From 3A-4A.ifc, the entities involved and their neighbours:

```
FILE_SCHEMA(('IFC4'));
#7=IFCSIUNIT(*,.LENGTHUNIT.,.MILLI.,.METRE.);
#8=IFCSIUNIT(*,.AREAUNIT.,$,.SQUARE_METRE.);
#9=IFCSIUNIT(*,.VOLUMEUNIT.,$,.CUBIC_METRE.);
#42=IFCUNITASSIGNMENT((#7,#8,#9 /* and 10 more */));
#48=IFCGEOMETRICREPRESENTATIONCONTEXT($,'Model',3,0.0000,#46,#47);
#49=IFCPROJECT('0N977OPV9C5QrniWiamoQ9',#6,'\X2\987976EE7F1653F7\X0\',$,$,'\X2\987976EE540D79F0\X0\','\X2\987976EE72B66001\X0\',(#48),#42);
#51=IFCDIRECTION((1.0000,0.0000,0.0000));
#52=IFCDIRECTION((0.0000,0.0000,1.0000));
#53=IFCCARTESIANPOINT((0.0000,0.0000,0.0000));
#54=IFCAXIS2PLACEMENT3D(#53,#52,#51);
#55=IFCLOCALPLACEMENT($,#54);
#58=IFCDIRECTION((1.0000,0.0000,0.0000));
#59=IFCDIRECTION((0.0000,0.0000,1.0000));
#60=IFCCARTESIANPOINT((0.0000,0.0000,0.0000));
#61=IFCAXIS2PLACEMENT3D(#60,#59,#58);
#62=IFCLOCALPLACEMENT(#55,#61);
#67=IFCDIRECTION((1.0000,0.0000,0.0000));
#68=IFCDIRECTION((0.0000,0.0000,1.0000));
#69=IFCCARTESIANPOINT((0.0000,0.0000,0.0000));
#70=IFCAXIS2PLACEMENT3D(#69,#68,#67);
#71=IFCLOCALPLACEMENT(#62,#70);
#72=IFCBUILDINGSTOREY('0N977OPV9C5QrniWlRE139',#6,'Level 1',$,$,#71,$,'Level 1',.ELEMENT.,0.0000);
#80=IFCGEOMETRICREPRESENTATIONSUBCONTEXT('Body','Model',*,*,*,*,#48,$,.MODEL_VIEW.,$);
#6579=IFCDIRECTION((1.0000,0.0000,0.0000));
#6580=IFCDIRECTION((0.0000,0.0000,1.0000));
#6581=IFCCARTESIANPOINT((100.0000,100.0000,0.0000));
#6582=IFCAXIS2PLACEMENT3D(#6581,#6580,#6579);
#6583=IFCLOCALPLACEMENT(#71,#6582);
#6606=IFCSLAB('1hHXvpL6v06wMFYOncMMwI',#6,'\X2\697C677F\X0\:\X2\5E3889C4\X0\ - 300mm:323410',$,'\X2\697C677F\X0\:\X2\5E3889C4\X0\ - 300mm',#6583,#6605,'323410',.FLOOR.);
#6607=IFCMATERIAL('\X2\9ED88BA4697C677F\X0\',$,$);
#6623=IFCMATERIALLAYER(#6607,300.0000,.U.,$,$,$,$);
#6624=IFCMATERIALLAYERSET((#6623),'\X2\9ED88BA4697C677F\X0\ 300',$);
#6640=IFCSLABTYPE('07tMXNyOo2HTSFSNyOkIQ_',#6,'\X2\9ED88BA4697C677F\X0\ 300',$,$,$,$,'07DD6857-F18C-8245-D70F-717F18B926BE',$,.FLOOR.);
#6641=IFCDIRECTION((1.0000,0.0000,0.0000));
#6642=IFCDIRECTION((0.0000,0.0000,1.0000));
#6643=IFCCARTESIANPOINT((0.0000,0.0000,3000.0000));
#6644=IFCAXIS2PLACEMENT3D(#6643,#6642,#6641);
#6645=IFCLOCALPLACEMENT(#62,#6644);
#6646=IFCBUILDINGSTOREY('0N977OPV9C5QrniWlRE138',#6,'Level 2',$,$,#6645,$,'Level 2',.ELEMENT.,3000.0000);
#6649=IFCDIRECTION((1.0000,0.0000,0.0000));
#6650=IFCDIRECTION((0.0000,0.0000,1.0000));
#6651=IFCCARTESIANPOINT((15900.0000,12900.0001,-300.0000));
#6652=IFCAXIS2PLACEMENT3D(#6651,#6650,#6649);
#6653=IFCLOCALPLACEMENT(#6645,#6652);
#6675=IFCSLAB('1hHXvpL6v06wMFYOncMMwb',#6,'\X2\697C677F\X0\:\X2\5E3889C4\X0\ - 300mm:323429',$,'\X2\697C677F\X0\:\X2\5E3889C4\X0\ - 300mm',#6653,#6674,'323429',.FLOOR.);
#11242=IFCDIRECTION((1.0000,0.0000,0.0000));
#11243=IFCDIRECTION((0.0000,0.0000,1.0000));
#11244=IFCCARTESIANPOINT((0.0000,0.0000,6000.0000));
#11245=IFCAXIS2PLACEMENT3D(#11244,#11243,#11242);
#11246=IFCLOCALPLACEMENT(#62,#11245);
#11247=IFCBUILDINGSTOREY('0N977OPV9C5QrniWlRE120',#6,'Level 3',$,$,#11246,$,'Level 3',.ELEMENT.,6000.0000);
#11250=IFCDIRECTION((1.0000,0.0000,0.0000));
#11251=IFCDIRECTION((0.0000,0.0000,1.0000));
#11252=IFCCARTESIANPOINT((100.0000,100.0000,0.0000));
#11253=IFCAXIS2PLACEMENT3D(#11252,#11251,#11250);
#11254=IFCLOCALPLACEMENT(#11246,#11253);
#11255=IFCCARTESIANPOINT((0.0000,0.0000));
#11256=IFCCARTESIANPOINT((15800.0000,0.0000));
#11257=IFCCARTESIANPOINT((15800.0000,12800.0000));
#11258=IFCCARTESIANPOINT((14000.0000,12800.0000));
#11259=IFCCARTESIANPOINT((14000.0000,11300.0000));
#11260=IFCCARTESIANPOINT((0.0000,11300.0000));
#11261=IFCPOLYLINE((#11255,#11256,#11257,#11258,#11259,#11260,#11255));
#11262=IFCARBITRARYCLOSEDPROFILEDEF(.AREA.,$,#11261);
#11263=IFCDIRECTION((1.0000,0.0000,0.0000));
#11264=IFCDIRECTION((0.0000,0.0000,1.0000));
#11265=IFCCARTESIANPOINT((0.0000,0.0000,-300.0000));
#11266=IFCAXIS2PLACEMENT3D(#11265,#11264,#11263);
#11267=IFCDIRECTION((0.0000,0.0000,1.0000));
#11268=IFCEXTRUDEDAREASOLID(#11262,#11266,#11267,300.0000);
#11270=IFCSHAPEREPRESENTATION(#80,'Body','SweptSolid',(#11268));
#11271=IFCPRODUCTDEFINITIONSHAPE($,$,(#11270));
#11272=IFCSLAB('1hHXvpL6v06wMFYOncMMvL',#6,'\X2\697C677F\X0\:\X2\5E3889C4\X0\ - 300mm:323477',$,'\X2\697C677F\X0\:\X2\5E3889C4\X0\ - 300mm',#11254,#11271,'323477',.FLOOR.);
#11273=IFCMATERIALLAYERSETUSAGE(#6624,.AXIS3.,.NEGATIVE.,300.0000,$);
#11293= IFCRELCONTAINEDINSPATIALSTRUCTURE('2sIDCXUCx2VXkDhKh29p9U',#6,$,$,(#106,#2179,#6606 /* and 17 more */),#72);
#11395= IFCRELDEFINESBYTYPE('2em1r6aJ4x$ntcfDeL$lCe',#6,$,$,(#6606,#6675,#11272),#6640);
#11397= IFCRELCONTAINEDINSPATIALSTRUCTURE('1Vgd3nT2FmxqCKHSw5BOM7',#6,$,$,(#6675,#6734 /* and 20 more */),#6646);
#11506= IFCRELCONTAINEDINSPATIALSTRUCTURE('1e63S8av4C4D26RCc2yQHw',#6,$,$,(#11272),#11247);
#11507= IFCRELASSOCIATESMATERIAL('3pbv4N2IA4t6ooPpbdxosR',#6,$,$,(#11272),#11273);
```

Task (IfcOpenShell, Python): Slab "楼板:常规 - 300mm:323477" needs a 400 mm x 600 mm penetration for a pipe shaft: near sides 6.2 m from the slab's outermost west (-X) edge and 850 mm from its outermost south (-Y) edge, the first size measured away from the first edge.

```python
import numpy as np
import ifcopenshell
import ifcopenshell.api.feature
import ifcopenshell.api.geometry
import ifcopenshell.api.root
import ifcopenshell.geom
import ifcopenshell.util.placement
import ifcopenshell.util.representation
import ifcopenshell.util.shape
import ifcopenshell.util.unit

model = ifcopenshell.open("3A-4A.ifc")
unit_scale = ifcopenshell.util.unit.calculate_unit_scale(model)
settings = ifcopenshell.geom.settings()


def volume(element):
    """Net volume in cubic metres, openings subtracted."""
    shape = ifcopenshell.geom.create_shape(settings, element)
    return ifcopenshell.util.shape.get_volume(shape.geometry)


slab = model.by_id(11272)
before = volume(slab)

# Extent in the slab's own axes, in metres. The edges named are its -X and -Y sides.
slab_shape = ifcopenshell.geom.create_shape(settings, slab)
vertices = ifcopenshell.util.shape.get_vertices(slab_shape.geometry)
x_min, y_min, bottom = vertices.min(axis=0)
top = vertices[:, 2].max()

opening = ifcopenshell.api.root.create_entity(model, ifc_class="IfcOpeningElement", name="Pipe shaft opening", predefined_type="OPENING")
context = ifcopenshell.util.representation.get_context(model, "Model", "Body", "MODEL_VIEW")
width, depth = 0.4, 0.6
outline = [(0.0, 0.0), (width, 0.0), (width, depth), (0.0, depth), (0.0, 0.0)]
# Overshoot both faces by 50 mm so the cut is clean.
shape = ifcopenshell.api.geometry.add_slab_representation(
    model, context=context, depth=top - bottom + 0.1, polyline=outline
)
ifcopenshell.api.geometry.assign_representation(model, product=opening, representation=shape)

matrix = ifcopenshell.util.placement.get_local_placement(slab.ObjectPlacement)
matrix[:, 3] = matrix @ np.append(np.array([x_min + 6.2, y_min + 0.85, bottom - 0.05]) / unit_scale, 1.0)
ifcopenshell.api.geometry.edit_object_placement(model, product=opening, matrix=matrix, is_si=False)
ifcopenshell.api.feature.add_feature(model, feature=opening, element=slab)

after = volume(slab)

print(f"slab volume {before:.3f} -> {after:.3f} m3")

model.write("3A-4A_edited.ifc")
```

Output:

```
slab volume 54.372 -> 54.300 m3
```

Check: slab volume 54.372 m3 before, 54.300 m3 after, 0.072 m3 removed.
